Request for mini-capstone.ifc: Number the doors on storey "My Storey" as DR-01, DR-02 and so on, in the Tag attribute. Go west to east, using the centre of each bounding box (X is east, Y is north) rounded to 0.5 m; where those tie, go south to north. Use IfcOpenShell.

First a look at what the model holds.

```python
import ifcopenshell
import ifcopenshell.util.element
import ifcopenshell.util.placement

model = ifcopenshell.open("mini-capstone.ifc")
print(model.schema)
storey = next(s for s in model.by_type("IfcBuildingStorey") if s.Name == "My Storey")
doors = [e for e in ifcopenshell.util.element.get_decomposition(storey) if e.is_a("IfcDoor")]
for e in sorted(doors, key=lambda e: e.id()):
    origin = ifcopenshell.util.placement.get_local_placement(e.ObjectPlacement)[:3, 3]
    print(e.id(), e.Tag, e.Name, origin.round(2) + 0.0, sep=" | ")
```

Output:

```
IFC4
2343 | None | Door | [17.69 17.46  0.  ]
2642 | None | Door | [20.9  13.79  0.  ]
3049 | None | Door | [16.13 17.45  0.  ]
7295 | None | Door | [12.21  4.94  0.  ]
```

```python
import ifcopenshell
import ifcopenshell.geom
import ifcopenshell.util.element
import ifcopenshell.util.shape

model = ifcopenshell.open("mini-capstone.ifc")
settings = ifcopenshell.geom.settings()
settings.set("use-world-coords", True)


def centre(element):
    shape = ifcopenshell.geom.create_shape(settings, element)
    return ifcopenshell.util.shape.get_bbox_centroid(shape.geometry)


storey = next(s for s in model.by_type("IfcBuildingStorey") if s.Name == "My Storey")
doors = [e for e in ifcopenshell.util.element.get_decomposition(storey) if e.is_a("IfcDoor")]

# Insertion points can sit at a corner or the storey origin, so sort by the geometry (in metres).
centres = {e: centre(e) for e in doors}
doors.sort(key=lambda e: (round(centres[e][0] / 0.5), centres[e][1]))

for i, e in enumerate(doors, start=1):
    number = f"DR-{i:02d}"
    e.Tag = number
    print(e.id(), number)

model.write("mini-capstone_edited.ifc")
```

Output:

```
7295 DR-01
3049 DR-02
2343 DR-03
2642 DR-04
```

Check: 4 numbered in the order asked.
